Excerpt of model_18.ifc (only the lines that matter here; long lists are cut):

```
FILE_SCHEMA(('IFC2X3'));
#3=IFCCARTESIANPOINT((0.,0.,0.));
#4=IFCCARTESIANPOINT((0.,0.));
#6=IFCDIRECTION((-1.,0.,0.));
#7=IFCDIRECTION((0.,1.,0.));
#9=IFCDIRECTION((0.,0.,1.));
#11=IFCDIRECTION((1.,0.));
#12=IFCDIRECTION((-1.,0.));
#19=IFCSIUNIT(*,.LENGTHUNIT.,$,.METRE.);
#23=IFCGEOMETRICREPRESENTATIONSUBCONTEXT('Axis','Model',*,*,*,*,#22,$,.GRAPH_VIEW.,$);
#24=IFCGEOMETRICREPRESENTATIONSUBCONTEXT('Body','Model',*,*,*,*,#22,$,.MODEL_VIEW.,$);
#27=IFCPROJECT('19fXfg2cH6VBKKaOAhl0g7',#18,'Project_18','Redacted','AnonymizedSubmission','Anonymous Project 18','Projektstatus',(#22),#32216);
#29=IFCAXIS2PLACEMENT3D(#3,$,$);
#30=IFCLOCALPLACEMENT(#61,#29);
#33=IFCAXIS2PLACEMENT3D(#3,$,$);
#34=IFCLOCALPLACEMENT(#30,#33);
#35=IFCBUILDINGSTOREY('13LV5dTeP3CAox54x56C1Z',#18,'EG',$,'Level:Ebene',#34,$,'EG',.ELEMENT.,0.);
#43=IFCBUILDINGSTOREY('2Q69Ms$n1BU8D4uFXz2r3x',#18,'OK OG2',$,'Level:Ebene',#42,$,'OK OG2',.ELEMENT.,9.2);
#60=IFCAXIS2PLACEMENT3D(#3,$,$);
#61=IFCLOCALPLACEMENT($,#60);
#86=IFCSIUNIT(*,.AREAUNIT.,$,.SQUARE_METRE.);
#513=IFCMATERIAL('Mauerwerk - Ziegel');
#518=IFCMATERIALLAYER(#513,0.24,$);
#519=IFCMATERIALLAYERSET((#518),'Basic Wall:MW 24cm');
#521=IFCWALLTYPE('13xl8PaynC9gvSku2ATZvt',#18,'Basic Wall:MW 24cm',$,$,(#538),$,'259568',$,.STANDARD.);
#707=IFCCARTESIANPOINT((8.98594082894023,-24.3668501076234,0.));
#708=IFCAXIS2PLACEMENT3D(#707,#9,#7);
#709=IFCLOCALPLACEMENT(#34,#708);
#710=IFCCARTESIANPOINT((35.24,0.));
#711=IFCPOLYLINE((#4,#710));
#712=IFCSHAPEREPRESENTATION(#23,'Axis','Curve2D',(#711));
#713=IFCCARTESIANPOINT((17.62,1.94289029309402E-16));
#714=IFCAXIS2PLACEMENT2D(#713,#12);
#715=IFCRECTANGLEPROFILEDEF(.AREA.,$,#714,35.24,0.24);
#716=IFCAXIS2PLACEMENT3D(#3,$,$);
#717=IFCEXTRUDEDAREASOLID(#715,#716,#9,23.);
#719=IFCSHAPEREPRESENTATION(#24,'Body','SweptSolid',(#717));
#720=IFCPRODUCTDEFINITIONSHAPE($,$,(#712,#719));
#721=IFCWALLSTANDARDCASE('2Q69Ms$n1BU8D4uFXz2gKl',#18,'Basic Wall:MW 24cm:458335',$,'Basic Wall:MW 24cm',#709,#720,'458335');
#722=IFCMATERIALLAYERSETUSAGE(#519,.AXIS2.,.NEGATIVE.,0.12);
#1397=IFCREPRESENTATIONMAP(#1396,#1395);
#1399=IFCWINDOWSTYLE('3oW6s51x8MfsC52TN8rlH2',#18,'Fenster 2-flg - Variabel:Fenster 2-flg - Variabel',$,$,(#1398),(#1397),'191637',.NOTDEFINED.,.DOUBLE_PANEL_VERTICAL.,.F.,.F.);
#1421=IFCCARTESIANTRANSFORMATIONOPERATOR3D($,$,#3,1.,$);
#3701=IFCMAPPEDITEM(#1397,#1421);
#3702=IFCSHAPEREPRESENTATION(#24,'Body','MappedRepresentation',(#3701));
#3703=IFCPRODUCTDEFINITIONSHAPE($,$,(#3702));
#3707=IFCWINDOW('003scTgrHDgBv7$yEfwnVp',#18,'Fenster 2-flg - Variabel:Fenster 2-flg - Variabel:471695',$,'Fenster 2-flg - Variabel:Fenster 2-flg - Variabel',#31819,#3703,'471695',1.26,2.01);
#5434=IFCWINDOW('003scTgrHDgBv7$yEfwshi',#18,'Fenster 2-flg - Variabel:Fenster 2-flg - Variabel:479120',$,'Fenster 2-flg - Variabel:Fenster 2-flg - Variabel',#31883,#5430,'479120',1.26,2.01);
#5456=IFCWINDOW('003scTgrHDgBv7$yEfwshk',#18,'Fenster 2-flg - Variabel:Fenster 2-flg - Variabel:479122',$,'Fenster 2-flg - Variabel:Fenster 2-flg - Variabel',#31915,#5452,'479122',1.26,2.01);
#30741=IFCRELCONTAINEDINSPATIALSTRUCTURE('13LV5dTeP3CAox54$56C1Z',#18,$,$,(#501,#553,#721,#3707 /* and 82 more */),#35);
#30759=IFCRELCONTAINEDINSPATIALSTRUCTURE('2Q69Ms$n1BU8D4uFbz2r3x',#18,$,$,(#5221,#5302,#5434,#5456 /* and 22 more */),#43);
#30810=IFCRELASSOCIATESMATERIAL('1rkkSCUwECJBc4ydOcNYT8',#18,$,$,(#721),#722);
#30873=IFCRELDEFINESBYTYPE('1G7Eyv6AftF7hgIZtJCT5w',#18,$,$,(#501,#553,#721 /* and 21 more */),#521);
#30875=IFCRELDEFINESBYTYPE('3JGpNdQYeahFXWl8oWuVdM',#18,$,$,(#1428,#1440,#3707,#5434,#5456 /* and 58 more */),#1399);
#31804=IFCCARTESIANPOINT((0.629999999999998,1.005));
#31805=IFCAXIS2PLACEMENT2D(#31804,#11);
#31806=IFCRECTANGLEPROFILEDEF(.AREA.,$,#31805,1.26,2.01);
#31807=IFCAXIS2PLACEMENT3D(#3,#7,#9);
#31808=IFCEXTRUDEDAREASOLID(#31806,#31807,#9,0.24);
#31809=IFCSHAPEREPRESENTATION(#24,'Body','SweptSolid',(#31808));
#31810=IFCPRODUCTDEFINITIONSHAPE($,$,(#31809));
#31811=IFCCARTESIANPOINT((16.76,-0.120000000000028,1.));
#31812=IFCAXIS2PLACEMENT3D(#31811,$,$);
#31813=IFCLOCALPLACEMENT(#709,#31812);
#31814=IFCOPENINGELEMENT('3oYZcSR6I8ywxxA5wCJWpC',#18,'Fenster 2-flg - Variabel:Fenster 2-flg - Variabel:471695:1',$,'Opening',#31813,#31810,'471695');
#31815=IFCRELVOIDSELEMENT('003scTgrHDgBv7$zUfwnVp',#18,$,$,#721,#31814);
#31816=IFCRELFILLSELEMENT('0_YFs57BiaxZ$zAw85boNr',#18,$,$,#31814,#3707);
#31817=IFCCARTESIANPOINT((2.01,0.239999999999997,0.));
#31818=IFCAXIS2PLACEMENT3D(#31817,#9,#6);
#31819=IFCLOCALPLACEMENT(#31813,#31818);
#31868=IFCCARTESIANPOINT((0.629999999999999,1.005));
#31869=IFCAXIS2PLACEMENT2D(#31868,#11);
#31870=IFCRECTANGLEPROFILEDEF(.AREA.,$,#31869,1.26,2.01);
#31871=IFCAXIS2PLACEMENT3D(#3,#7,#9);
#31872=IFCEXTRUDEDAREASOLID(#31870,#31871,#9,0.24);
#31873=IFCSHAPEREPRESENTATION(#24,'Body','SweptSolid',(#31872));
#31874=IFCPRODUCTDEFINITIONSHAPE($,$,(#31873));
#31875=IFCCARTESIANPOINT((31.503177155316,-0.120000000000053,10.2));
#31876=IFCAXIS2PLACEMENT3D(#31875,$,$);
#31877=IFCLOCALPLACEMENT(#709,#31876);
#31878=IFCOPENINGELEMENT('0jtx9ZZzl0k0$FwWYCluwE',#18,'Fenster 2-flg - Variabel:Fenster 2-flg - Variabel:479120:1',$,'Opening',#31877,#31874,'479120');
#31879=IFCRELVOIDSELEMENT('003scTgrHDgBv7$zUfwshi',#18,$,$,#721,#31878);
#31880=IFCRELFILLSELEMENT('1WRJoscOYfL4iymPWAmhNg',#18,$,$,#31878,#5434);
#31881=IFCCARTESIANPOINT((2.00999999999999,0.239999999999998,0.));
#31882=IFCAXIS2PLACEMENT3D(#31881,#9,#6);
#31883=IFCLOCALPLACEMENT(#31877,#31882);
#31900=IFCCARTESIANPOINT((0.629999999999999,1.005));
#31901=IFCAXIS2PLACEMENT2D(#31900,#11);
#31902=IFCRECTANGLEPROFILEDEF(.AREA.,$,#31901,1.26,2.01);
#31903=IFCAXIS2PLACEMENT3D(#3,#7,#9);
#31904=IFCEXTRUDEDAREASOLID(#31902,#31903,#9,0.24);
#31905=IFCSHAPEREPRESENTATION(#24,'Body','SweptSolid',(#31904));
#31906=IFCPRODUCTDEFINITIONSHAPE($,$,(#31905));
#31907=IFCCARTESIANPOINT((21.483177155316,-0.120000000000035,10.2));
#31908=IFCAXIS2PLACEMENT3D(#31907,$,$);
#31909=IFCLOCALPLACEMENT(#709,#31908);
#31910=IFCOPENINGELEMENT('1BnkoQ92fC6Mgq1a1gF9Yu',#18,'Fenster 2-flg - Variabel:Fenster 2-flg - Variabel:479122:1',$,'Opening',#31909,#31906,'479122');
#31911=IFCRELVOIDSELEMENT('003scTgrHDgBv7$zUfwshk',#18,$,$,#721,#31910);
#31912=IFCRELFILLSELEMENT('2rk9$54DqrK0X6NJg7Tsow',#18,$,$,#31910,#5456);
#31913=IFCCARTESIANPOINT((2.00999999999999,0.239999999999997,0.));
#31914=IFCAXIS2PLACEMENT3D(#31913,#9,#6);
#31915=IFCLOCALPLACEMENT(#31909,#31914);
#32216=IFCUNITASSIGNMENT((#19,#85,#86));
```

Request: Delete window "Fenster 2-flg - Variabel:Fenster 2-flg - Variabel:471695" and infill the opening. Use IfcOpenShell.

```python
import ifcopenshell
import ifcopenshell.api.feature
import ifcopenshell.api.root
import ifcopenshell.geom
import ifcopenshell.util.shape

model = ifcopenshell.open("model_18.ifc")
settings = ifcopenshell.geom.settings()


def volume(element):
    """Net volume in cubic metres, openings subtracted."""
    shape = ifcopenshell.geom.create_shape(settings, element)
    return ifcopenshell.util.shape.get_volume(shape.geometry)


window = model.by_id(3707)
opening = window.FillsVoids[0].RelatingOpeningElement
wall = opening.VoidsElements[0].RelatingBuildingElement
before = volume(wall)

ifcopenshell.api.root.remove_product(model, product=window)
ifcopenshell.api.feature.remove_feature(model, feature=opening)

after = volume(wall)

print(f"wall volume {before:.3f} -> {after:.3f} m3")

model.write("model_18-out.ifc")
```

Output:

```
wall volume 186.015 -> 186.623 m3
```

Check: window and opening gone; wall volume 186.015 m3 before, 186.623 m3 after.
